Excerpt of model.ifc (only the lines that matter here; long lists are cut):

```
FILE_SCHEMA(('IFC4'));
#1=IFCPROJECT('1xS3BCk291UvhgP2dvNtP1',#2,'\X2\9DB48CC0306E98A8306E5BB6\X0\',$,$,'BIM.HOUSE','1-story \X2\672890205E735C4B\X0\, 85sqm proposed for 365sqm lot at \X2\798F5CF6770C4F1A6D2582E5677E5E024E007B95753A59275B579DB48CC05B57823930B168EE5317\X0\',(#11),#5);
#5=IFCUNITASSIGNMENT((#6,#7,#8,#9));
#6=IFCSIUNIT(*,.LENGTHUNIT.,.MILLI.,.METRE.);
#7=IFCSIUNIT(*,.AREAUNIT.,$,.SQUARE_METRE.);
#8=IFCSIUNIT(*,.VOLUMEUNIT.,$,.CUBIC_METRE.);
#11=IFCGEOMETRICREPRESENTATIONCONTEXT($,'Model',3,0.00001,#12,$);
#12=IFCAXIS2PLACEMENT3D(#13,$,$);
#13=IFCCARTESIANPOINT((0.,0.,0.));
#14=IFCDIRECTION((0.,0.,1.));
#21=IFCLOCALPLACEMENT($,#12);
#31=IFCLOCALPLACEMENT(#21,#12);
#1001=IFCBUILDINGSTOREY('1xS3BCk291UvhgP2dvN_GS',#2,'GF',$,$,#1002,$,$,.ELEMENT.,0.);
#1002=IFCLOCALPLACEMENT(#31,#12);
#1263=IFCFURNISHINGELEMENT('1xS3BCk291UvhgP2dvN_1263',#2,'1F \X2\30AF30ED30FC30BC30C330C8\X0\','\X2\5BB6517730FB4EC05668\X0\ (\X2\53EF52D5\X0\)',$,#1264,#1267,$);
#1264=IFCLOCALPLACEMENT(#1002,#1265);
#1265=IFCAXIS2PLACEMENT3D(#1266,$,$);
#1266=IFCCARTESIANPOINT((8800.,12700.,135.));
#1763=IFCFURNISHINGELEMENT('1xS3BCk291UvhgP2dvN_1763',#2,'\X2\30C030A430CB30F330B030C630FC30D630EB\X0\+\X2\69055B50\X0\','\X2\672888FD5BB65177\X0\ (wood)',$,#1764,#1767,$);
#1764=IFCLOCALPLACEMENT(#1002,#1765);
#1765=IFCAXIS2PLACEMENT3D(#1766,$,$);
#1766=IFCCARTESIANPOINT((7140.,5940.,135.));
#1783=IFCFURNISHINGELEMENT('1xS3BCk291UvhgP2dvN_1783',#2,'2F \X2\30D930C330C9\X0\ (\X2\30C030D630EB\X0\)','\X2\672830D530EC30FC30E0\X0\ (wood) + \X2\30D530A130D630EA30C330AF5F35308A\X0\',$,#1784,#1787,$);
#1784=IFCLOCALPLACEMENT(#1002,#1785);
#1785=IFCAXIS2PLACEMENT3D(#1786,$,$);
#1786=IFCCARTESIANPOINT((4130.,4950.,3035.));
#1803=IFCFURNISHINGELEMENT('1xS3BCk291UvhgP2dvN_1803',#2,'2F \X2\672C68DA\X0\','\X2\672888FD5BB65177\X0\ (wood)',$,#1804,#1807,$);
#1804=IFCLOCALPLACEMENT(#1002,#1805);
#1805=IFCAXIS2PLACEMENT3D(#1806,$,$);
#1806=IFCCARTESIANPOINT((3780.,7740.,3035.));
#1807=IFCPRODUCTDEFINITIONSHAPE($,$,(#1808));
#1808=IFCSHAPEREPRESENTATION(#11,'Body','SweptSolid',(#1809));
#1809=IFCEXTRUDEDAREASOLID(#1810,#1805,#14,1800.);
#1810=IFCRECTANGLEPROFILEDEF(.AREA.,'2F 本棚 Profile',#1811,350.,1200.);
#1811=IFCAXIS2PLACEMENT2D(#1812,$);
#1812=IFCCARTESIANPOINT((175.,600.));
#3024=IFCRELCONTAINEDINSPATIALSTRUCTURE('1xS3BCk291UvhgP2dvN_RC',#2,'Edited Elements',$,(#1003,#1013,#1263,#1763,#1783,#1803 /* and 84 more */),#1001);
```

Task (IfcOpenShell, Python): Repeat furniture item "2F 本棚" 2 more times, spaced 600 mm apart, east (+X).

```python
import numpy as np
import ifcopenshell
import ifcopenshell.api.geometry
import ifcopenshell.api.root
import ifcopenshell.util.element
import ifcopenshell.util.placement
import ifcopenshell.util.unit

model = ifcopenshell.open("model.ifc")
unit_scale = ifcopenshell.util.unit.calculate_unit_scale(model)


def reuse_history(source, copy):
    """copy_class also copies each property set's owner history, people and application; keep the originals."""
    for rel in copy.IsDefinedBy:
        if rel.is_a("IfcRelDefinesByProperties") and (history := rel.RelatingPropertyDefinition.OwnerHistory):
            rel.RelatingPropertyDefinition.OwnerHistory = source.OwnerHistory
            ifcopenshell.util.element.remove_deep2(model, history)


source = model.by_guid("1xS3BCk291UvhgP2dvN_1803")
base = ifcopenshell.util.placement.get_local_placement(source.ObjectPlacement)
step = np.array([1.0, 0.0, 0.0]) * 0.6 / unit_scale

for i in range(1, 3):
    copy = ifcopenshell.api.root.copy_class(model, product=source)
    copy.Representation = ifcopenshell.util.element.copy_deep(
        model, source.Representation, exclude=["IfcGeometricRepresentationContext", "IfcRepresentationMap"]
    )
    reuse_history(source, copy)
    matrix = base.copy()
    matrix[:3, 3] += i * step
    print("added at", matrix[:3, 3].round(3) + 0.0)
    ifcopenshell.api.geometry.edit_object_placement(model, product=copy, matrix=matrix, is_si=False)

model.write("model_updated.ifc")
```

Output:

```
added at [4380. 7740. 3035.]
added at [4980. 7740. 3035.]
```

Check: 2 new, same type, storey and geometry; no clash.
